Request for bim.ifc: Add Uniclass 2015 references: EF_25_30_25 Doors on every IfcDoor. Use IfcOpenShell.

First a look at what the model holds.

```python
import ifcopenshell

model = ifcopenshell.open("bim.ifc")
print(model.schema)
print("classifications:", [c.Name for c in model.by_type("IfcClassification")])
for ifc_class in ("IfcDoor", "IfcRoof", "IfcStair", "IfcWall", "IfcWindow"):
    print(ifc_class, len(model.by_type(ifc_class)))
```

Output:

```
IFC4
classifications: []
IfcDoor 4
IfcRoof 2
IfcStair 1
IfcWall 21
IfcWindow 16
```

```python
import ifcopenshell
import ifcopenshell.api.classification

model = ifcopenshell.open("bim.ifc")

system = ifcopenshell.api.classification.add_classification(model, classification="Uniclass 2015")

codes = {
    "IfcDoor": ("EF_25_30_25", "Doors"),
}
for ifc_class, (code, name) in codes.items():
    products = model.by_type(ifc_class)
    ifcopenshell.api.classification.add_reference(
        model, products=products, classification=system, identification=code, name=name
    )
    print(code, len(products))

model.write("bim_edited.ifc")
```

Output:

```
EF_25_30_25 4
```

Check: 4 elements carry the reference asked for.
